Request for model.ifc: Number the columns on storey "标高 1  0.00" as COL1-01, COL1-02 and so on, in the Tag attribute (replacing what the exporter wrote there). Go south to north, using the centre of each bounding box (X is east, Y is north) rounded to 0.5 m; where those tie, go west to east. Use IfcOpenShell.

First a look at what the model holds.

```python
import ifcopenshell
import ifcopenshell.util.element
import ifcopenshell.util.placement

model = ifcopenshell.open("model.ifc")
print(model.schema)
storey = next(s for s in model.by_type("IfcBuildingStorey") if s.Name == "标高 1  0.00")
columns = [e for e in ifcopenshell.util.element.get_decomposition(storey) if e.is_a("IfcColumn")]
for e in sorted(columns, key=lambda e: e.id()):
    origin = ifcopenshell.util.placement.get_local_placement(e.ObjectPlacement)[:3, 3]
    print(e.id(), e.Tag, e.Name, origin.round(2) + 0.0, sep=" | ")
```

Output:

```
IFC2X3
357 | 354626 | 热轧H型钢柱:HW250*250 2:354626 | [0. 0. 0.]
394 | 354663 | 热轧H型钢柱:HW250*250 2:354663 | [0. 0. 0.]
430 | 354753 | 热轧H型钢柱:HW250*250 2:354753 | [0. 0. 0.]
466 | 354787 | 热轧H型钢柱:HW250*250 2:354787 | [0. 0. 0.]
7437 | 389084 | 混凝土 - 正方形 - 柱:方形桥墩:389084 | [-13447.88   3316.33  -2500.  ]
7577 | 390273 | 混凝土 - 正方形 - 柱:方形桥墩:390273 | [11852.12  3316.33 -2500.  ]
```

```python
import ifcopenshell
import ifcopenshell.geom
import ifcopenshell.util.element
import ifcopenshell.util.shape

model = ifcopenshell.open("model.ifc")
settings = ifcopenshell.geom.settings()
settings.set("use-world-coords", True)


def centre(element):
    shape = ifcopenshell.geom.create_shape(settings, element)
    return ifcopenshell.util.shape.get_bbox_centroid(shape.geometry)


storey = next(s for s in model.by_type("IfcBuildingStorey") if s.Name == "标高 1  0.00")
columns = [e for e in ifcopenshell.util.element.get_decomposition(storey) if e.is_a("IfcColumn")]

# Insertion points can sit at a corner or the storey origin, so sort by the geometry (in metres).
centres = {e: centre(e) for e in columns}
columns.sort(key=lambda e: (round(centres[e][1] / 0.5), centres[e][0]))

for i, e in enumerate(columns, start=1):
    number = f"COL1-{i:02d}"
    e.Tag = number
    print(e.id(), number)

model.write("model_updated.ifc")
```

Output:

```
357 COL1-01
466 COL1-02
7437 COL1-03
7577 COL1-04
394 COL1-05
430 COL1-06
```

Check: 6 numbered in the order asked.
